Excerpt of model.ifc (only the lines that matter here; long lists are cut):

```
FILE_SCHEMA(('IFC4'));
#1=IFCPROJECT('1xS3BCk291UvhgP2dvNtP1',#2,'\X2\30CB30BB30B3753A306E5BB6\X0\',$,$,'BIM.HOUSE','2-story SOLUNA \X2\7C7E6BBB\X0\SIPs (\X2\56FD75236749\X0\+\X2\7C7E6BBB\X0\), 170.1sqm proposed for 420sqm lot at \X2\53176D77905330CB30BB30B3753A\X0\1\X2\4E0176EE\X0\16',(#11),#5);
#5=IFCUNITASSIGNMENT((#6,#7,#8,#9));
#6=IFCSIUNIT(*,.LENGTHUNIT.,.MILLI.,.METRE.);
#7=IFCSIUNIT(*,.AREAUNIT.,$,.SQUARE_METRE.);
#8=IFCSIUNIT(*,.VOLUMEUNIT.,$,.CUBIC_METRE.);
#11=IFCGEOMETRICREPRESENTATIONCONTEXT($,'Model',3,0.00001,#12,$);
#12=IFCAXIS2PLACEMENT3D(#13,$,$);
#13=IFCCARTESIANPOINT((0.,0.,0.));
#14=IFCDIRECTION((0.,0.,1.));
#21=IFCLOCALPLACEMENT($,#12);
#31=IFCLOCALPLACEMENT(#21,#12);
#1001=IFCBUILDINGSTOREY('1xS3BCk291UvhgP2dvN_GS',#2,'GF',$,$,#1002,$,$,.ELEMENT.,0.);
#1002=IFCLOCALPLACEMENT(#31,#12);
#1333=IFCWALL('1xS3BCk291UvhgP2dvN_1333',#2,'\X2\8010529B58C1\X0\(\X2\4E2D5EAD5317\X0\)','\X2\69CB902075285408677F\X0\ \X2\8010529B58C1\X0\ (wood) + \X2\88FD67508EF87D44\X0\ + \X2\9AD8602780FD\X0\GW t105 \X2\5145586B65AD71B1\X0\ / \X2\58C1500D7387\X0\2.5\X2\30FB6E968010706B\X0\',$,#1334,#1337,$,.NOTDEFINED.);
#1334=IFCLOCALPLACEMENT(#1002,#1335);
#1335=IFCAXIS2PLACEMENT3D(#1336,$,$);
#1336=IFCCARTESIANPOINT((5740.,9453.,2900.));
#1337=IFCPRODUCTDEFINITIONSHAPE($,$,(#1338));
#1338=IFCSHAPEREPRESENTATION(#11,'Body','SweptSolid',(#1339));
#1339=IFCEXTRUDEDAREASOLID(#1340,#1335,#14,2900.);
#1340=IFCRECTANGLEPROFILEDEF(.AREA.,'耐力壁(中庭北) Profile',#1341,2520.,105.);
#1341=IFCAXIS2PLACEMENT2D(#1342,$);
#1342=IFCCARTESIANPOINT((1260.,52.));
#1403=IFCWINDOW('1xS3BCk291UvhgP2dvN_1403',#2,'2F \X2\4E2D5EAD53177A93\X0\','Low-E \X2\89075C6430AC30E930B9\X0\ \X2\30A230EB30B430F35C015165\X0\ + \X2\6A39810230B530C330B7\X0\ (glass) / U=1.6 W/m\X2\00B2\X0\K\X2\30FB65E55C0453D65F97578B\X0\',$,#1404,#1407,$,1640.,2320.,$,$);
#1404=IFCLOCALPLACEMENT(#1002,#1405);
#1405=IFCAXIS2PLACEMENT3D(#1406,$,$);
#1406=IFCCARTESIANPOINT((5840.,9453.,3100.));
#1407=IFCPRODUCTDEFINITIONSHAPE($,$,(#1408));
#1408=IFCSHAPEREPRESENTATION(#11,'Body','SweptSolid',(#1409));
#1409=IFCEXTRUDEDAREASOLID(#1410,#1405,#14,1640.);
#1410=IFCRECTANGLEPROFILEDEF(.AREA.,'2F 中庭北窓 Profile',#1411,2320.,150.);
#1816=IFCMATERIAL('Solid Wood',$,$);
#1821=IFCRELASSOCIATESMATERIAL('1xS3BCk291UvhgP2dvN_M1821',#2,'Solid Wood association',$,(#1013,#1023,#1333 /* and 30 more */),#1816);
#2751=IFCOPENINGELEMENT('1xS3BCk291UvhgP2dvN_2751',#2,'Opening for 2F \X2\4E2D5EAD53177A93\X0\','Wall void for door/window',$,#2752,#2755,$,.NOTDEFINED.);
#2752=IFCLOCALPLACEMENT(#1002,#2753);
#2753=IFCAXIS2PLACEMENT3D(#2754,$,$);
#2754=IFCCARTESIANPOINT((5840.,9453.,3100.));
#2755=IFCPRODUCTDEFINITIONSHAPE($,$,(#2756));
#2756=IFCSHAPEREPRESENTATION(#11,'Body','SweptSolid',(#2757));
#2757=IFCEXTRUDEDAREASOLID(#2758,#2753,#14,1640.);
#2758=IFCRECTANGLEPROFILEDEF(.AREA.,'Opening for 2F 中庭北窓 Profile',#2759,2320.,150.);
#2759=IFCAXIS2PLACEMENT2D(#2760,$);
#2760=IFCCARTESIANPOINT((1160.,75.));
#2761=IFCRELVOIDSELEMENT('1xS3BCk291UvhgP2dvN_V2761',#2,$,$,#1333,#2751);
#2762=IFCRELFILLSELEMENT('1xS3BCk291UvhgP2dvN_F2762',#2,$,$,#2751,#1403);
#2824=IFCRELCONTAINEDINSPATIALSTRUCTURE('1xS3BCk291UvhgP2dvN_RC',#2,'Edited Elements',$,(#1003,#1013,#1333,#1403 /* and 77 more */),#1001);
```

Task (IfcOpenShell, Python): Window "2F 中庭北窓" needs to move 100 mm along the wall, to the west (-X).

```python
import ifcopenshell
import ifcopenshell.api.geometry
import ifcopenshell.util.placement
import ifcopenshell.util.unit

model = ifcopenshell.open("model.ifc")
unit_scale = ifcopenshell.util.unit.calculate_unit_scale(model)

window = model.by_guid("1xS3BCk291UvhgP2dvN_1403")
opening = window.FillsVoids[0].RelatingOpeningElement
wall = opening.VoidsElements[0].RelatingBuildingElement

wall_matrix = ifcopenshell.util.placement.get_local_placement(wall.ObjectPlacement)
shift = wall_matrix[:3, 0] * -0.1 / unit_scale
before = ifcopenshell.util.placement.get_local_placement(window.ObjectPlacement)[:3, 3].copy()

# The window is not placed relative to its opening, so move both.
for product in (opening, window):
    matrix = ifcopenshell.util.placement.get_local_placement(product.ObjectPlacement)
    matrix[:3, 3] += shift
    ifcopenshell.api.geometry.edit_object_placement(model, product=product, matrix=matrix, is_si=False)

after = ifcopenshell.util.placement.get_local_placement(window.ObjectPlacement)[:3, 3]
print("window moved by", (after - before).round(3) + 0.0)

model.write("model_rev.ifc")
```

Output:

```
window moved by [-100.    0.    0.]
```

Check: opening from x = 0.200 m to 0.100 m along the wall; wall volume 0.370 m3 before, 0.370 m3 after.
